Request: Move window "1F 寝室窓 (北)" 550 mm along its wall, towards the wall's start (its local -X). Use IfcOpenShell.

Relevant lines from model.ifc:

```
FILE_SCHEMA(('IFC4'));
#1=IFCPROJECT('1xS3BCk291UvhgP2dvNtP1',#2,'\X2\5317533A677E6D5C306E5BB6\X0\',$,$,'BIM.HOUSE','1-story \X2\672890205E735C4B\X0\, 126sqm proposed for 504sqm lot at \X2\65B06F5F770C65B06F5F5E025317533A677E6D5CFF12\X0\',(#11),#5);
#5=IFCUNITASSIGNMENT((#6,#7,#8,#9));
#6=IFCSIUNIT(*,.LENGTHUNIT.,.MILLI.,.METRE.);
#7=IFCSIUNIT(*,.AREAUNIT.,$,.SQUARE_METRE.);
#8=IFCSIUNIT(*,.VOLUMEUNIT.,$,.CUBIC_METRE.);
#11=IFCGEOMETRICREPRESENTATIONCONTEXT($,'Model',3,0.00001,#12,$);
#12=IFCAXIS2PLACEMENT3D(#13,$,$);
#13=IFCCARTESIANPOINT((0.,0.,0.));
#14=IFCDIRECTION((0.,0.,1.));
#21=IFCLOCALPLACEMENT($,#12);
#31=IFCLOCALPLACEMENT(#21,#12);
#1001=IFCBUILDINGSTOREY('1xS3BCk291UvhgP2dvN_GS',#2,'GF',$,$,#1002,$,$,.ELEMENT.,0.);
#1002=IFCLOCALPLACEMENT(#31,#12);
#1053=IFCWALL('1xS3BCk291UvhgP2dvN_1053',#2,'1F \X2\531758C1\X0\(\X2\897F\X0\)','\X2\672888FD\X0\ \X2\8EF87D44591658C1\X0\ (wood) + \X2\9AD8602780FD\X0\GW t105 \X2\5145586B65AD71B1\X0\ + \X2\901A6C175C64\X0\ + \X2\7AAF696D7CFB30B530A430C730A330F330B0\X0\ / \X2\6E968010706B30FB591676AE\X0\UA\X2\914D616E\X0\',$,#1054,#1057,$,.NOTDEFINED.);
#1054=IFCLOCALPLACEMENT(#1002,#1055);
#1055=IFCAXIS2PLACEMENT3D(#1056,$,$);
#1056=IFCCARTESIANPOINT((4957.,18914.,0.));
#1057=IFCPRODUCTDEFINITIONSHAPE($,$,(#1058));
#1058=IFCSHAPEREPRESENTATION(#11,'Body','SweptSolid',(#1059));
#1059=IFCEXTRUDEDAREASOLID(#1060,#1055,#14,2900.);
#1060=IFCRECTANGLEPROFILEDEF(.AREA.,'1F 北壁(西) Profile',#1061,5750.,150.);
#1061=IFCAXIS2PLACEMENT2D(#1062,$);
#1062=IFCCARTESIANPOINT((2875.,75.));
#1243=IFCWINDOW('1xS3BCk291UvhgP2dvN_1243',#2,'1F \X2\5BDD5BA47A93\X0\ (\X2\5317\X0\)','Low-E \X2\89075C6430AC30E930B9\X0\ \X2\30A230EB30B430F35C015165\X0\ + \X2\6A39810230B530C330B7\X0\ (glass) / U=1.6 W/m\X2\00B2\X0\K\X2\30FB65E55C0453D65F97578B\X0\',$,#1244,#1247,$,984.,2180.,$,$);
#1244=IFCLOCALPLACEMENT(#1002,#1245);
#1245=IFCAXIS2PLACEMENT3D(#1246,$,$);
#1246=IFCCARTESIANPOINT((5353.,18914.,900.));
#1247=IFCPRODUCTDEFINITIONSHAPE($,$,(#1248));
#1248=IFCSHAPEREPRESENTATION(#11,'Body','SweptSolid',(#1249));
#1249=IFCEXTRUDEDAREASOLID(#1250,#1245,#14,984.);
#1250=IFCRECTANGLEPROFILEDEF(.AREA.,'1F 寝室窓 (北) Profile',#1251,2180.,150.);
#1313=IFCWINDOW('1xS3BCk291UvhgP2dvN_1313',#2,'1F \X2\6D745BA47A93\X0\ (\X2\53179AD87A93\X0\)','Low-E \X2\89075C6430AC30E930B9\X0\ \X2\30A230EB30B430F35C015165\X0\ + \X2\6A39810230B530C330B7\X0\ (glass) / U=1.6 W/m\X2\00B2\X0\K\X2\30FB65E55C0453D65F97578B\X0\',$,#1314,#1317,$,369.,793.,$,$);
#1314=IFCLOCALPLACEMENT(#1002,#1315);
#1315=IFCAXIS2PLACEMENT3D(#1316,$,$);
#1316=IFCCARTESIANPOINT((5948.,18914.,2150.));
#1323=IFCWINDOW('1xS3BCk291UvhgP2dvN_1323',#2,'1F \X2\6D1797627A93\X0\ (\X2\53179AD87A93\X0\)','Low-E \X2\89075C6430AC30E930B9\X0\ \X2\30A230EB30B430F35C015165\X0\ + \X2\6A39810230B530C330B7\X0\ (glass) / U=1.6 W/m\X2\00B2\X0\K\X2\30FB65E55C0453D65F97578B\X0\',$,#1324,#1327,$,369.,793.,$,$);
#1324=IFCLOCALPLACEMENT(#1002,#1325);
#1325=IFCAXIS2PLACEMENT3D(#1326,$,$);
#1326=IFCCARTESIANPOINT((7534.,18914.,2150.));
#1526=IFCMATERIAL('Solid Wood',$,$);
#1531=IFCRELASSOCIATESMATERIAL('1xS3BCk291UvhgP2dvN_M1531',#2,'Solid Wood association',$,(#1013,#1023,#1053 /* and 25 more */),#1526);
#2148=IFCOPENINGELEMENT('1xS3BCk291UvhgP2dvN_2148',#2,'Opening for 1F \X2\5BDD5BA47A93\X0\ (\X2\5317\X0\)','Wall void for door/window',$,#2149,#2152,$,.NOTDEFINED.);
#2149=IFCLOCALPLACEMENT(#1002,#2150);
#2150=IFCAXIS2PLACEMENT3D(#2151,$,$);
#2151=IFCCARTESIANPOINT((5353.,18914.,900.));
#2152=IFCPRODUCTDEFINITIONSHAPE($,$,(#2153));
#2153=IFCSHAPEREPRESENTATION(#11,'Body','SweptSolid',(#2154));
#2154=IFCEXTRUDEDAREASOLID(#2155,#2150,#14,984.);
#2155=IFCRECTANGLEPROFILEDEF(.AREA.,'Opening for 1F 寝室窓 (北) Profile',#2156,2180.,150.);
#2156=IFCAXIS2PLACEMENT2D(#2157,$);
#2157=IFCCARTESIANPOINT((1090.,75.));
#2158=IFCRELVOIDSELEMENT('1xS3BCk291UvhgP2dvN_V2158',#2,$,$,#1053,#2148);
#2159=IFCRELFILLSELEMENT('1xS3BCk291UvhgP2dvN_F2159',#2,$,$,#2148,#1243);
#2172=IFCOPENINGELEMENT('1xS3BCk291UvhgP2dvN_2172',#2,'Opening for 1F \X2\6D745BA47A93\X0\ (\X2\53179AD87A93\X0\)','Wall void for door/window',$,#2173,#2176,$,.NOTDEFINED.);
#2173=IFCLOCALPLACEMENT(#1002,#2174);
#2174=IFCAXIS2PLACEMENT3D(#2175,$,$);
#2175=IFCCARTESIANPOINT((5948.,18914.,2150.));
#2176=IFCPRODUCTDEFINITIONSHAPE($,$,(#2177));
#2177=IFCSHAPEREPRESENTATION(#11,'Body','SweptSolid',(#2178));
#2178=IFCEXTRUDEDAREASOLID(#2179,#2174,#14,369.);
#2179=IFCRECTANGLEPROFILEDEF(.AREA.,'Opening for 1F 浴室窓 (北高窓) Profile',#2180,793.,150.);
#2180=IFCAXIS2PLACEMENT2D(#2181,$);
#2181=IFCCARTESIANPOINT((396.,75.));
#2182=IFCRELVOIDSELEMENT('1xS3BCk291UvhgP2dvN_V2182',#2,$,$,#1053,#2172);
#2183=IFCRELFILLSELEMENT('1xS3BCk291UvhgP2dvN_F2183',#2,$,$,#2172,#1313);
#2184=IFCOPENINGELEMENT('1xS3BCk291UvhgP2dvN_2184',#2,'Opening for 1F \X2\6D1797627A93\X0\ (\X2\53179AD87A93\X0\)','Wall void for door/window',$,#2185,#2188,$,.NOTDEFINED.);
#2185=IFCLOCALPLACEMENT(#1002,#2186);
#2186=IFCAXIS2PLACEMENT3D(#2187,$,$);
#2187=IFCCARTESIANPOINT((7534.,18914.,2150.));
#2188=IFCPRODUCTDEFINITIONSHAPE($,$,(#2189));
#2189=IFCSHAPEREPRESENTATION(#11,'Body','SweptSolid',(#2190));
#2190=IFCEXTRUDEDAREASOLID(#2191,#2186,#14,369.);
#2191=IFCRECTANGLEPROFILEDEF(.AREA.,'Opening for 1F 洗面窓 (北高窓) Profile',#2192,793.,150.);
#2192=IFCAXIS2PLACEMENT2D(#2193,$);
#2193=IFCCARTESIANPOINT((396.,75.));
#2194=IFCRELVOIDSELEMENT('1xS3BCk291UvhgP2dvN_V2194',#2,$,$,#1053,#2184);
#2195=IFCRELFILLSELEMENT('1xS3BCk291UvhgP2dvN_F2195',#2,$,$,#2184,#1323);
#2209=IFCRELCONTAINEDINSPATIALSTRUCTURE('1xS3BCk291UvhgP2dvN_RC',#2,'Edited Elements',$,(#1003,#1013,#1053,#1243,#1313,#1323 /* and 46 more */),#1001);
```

```python
import ifcopenshell
import ifcopenshell.api.geometry
import ifcopenshell.util.placement
import ifcopenshell.util.unit

model = ifcopenshell.open("model.ifc")
unit_scale = ifcopenshell.util.unit.calculate_unit_scale(model)

window = model.by_guid("1xS3BCk291UvhgP2dvN_1243")
opening = window.FillsVoids[0].RelatingOpeningElement
wall = opening.VoidsElements[0].RelatingBuildingElement

wall_matrix = ifcopenshell.util.placement.get_local_placement(wall.ObjectPlacement)
shift = wall_matrix[:3, 0] * -0.55 / unit_scale
before = ifcopenshell.util.placement.get_local_placement(window.ObjectPlacement)[:3, 3].copy()

# The window is not placed relative to its opening, so move both.
for product in (opening, window):
    matrix = ifcopenshell.util.placement.get_local_placement(product.ObjectPlacement)
    matrix[:3, 3] += shift
    ifcopenshell.api.geometry.edit_object_placement(model, product=product, matrix=matrix, is_si=False)

after = ifcopenshell.util.placement.get_local_placement(window.ObjectPlacement)[:3, 3]
print("window moved by", (after - before).round(3) + 0.0)

model.write("model_updated.ifc")
```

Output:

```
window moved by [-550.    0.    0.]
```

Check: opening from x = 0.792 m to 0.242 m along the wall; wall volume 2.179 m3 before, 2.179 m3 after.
